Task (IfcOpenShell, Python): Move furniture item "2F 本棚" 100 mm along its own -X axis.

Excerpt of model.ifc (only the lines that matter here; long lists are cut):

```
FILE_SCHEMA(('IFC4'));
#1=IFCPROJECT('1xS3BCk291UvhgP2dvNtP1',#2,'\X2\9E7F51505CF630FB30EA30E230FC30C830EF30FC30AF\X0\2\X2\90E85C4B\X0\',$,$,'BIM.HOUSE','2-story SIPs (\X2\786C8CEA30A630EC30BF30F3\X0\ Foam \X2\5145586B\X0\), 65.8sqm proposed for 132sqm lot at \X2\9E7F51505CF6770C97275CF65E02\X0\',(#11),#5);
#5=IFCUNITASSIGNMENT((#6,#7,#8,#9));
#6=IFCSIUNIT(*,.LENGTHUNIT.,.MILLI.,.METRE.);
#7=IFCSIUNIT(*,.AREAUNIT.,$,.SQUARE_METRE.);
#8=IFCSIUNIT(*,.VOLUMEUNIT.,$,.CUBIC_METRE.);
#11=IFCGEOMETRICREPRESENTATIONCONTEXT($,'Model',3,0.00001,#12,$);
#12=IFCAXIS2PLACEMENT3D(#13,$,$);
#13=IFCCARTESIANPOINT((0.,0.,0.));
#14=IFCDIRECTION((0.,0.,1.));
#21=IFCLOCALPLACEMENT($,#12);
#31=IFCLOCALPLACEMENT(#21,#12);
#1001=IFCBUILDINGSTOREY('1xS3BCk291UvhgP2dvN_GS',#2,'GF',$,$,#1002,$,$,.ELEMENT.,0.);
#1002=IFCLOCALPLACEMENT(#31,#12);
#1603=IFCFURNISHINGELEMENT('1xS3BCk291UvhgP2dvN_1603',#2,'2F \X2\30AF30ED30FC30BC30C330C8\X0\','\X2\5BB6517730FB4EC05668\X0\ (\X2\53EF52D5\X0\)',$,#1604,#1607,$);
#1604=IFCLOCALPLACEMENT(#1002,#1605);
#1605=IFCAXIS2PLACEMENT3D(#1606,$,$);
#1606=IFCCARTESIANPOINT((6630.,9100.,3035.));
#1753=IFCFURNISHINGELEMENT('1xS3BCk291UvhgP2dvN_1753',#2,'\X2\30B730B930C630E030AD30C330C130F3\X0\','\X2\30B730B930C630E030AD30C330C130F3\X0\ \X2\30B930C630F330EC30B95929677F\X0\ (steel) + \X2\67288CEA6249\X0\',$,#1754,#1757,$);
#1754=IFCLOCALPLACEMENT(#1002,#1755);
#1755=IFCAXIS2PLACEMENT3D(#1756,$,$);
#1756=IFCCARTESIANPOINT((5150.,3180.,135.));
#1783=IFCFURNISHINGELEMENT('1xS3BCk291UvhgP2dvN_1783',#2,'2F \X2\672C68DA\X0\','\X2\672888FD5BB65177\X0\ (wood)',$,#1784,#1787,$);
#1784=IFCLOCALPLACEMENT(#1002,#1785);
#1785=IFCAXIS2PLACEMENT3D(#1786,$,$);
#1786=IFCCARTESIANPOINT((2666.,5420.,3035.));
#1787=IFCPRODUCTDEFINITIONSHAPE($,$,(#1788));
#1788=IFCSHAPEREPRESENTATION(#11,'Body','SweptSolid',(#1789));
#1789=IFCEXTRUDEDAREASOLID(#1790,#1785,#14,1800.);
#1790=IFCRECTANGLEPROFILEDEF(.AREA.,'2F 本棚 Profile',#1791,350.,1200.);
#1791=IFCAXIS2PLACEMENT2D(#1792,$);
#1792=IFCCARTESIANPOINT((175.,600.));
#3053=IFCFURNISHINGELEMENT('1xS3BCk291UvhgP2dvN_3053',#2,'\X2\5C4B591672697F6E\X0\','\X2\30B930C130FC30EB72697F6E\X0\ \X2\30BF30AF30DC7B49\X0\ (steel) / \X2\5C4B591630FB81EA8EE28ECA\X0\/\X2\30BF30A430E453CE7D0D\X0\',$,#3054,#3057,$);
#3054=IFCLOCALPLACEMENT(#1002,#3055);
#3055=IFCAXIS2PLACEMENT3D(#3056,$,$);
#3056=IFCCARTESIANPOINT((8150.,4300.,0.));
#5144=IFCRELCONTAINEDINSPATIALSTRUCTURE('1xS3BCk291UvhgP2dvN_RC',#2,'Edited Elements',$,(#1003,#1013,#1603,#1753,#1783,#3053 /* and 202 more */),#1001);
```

```python
import ifcopenshell
import ifcopenshell.api.geometry
import ifcopenshell.util.placement

model = ifcopenshell.open("model.ifc")

item = model.by_guid("1xS3BCk291UvhgP2dvN_1783")
matrix = ifcopenshell.util.placement.get_local_placement(item.ObjectPlacement)
matrix[:3, 3] -= matrix[:3, 0] * 100.0
ifcopenshell.api.geometry.edit_object_placement(model, product=item, matrix=matrix, is_si=False)

print(ifcopenshell.util.placement.get_local_placement(item.ObjectPlacement).round(3) + 0.0)

model.write("model-out.ifc")
```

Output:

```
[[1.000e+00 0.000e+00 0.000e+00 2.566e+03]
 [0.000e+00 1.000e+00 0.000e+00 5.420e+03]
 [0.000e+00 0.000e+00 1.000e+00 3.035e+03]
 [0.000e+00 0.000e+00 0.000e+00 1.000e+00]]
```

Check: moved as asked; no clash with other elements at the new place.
